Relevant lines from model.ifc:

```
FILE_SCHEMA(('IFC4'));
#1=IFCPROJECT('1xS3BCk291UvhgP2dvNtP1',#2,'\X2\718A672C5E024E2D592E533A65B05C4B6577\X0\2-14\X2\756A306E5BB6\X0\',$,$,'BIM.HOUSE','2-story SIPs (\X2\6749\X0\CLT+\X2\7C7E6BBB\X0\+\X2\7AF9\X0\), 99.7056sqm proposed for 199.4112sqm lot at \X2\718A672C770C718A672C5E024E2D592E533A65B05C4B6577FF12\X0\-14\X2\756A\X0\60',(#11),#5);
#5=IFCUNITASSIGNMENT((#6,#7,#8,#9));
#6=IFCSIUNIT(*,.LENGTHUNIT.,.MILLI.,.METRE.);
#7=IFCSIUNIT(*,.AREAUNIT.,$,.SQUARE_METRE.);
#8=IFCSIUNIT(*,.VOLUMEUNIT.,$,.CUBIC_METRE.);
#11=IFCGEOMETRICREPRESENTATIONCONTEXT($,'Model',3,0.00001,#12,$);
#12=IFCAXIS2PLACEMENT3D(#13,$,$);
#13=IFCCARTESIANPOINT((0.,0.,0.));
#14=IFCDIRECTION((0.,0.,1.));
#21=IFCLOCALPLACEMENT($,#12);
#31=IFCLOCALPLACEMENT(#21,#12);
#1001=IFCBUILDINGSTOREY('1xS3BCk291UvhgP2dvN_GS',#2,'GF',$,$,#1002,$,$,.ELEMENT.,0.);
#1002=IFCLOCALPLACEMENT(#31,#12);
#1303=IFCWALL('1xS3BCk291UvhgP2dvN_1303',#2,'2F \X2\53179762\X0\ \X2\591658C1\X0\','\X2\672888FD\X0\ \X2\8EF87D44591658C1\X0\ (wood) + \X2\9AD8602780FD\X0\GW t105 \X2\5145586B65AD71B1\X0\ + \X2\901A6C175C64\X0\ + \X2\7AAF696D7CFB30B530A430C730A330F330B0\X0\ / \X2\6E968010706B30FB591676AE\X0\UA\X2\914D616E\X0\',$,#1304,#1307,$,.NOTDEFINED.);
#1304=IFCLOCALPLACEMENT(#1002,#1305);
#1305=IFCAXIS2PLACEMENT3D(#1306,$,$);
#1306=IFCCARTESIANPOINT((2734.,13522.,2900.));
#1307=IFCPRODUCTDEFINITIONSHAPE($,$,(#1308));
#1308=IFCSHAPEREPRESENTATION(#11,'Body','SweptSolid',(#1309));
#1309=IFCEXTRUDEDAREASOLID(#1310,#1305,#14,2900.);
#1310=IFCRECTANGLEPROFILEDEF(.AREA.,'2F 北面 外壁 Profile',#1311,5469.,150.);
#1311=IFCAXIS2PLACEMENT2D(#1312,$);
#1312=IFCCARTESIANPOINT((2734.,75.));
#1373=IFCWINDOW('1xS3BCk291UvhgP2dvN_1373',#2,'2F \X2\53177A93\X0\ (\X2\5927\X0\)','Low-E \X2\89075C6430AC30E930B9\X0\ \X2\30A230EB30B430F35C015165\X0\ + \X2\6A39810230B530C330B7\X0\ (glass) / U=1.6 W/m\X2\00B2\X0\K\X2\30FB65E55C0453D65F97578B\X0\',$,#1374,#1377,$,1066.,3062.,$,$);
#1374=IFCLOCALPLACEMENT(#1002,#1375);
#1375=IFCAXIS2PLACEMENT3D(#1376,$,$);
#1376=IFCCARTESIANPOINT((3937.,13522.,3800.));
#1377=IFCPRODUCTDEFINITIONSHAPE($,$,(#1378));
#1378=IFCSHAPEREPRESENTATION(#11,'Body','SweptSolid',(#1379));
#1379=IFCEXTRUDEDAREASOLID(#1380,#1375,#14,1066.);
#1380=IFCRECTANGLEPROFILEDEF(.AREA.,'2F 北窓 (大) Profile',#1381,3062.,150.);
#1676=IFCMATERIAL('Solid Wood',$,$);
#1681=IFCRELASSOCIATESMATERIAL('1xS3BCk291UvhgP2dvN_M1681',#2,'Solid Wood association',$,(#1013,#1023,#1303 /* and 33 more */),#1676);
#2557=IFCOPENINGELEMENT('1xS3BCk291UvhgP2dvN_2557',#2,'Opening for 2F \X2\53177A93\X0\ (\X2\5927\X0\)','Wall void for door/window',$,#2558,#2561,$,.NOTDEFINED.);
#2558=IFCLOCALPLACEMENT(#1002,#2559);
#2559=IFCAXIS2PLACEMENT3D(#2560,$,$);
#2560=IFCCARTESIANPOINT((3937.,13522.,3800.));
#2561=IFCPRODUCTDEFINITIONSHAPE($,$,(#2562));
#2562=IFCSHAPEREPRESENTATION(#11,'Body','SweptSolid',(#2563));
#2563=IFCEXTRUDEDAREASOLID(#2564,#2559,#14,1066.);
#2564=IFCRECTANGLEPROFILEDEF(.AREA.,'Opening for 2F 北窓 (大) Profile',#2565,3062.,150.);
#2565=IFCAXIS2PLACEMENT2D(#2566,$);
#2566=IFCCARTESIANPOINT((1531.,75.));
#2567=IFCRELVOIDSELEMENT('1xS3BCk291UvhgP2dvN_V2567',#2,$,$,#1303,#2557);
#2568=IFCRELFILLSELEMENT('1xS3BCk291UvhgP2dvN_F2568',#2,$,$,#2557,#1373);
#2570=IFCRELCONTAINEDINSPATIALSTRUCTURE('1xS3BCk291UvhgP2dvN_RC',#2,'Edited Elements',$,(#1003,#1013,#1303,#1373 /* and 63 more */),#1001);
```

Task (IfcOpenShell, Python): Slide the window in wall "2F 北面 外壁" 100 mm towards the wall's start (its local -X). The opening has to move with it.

```python
import ifcopenshell
import ifcopenshell.api.geometry
import ifcopenshell.util.placement

model = ifcopenshell.open("model.ifc")

window = model.by_guid("1xS3BCk291UvhgP2dvN_1373")
opening = window.FillsVoids[0].RelatingOpeningElement
wall = opening.VoidsElements[0].RelatingBuildingElement

wall_matrix = ifcopenshell.util.placement.get_local_placement(wall.ObjectPlacement)
shift = wall_matrix[:3, 0] * -100.0
before = ifcopenshell.util.placement.get_local_placement(window.ObjectPlacement)[:3, 3].copy()

# The window is not placed relative to its opening, so move both.
for product in (opening, window):
    matrix = ifcopenshell.util.placement.get_local_placement(product.ObjectPlacement)
    matrix[:3, 3] += shift
    ifcopenshell.api.geometry.edit_object_placement(model, product=product, matrix=matrix, is_si=False)

after = ifcopenshell.util.placement.get_local_placement(window.ObjectPlacement)[:3, 3]
print("window moved by", (after - before).round(3) + 0.0)

model.write("model_updated.ifc")
```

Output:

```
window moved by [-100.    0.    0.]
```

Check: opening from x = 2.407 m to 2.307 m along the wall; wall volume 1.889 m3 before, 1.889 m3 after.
